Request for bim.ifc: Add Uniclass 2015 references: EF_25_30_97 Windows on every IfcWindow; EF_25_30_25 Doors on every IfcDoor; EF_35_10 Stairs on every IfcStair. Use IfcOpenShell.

First a look at what the model holds.

```python
import ifcopenshell

model = ifcopenshell.open("bim.ifc")
print(model.schema)
print("classifications:", [c.Name for c in model.by_type("IfcClassification")])
for ifc_class in ("IfcDoor", "IfcRoof", "IfcStair", "IfcWall", "IfcWindow"):
    print(ifc_class, len(model.by_type(ifc_class)))
```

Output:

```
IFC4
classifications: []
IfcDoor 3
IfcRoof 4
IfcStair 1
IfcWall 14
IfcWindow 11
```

```python
import ifcopenshell
import ifcopenshell.api.classification

model = ifcopenshell.open("bim.ifc")

system = ifcopenshell.api.classification.add_classification(model, classification="Uniclass 2015")

codes = {
    "IfcWindow": ("EF_25_30_97", "Windows"),
    "IfcDoor": ("EF_25_30_25", "Doors"),
    "IfcStair": ("EF_35_10", "Stairs"),
}
for ifc_class, (code, name) in codes.items():
    products = model.by_type(ifc_class)
    ifcopenshell.api.classification.add_reference(
        model, products=products, classification=system, identification=code, name=name
    )
    print(code, len(products))

model.write("bim_updated.ifc")
```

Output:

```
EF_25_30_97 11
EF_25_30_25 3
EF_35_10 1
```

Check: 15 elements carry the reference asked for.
